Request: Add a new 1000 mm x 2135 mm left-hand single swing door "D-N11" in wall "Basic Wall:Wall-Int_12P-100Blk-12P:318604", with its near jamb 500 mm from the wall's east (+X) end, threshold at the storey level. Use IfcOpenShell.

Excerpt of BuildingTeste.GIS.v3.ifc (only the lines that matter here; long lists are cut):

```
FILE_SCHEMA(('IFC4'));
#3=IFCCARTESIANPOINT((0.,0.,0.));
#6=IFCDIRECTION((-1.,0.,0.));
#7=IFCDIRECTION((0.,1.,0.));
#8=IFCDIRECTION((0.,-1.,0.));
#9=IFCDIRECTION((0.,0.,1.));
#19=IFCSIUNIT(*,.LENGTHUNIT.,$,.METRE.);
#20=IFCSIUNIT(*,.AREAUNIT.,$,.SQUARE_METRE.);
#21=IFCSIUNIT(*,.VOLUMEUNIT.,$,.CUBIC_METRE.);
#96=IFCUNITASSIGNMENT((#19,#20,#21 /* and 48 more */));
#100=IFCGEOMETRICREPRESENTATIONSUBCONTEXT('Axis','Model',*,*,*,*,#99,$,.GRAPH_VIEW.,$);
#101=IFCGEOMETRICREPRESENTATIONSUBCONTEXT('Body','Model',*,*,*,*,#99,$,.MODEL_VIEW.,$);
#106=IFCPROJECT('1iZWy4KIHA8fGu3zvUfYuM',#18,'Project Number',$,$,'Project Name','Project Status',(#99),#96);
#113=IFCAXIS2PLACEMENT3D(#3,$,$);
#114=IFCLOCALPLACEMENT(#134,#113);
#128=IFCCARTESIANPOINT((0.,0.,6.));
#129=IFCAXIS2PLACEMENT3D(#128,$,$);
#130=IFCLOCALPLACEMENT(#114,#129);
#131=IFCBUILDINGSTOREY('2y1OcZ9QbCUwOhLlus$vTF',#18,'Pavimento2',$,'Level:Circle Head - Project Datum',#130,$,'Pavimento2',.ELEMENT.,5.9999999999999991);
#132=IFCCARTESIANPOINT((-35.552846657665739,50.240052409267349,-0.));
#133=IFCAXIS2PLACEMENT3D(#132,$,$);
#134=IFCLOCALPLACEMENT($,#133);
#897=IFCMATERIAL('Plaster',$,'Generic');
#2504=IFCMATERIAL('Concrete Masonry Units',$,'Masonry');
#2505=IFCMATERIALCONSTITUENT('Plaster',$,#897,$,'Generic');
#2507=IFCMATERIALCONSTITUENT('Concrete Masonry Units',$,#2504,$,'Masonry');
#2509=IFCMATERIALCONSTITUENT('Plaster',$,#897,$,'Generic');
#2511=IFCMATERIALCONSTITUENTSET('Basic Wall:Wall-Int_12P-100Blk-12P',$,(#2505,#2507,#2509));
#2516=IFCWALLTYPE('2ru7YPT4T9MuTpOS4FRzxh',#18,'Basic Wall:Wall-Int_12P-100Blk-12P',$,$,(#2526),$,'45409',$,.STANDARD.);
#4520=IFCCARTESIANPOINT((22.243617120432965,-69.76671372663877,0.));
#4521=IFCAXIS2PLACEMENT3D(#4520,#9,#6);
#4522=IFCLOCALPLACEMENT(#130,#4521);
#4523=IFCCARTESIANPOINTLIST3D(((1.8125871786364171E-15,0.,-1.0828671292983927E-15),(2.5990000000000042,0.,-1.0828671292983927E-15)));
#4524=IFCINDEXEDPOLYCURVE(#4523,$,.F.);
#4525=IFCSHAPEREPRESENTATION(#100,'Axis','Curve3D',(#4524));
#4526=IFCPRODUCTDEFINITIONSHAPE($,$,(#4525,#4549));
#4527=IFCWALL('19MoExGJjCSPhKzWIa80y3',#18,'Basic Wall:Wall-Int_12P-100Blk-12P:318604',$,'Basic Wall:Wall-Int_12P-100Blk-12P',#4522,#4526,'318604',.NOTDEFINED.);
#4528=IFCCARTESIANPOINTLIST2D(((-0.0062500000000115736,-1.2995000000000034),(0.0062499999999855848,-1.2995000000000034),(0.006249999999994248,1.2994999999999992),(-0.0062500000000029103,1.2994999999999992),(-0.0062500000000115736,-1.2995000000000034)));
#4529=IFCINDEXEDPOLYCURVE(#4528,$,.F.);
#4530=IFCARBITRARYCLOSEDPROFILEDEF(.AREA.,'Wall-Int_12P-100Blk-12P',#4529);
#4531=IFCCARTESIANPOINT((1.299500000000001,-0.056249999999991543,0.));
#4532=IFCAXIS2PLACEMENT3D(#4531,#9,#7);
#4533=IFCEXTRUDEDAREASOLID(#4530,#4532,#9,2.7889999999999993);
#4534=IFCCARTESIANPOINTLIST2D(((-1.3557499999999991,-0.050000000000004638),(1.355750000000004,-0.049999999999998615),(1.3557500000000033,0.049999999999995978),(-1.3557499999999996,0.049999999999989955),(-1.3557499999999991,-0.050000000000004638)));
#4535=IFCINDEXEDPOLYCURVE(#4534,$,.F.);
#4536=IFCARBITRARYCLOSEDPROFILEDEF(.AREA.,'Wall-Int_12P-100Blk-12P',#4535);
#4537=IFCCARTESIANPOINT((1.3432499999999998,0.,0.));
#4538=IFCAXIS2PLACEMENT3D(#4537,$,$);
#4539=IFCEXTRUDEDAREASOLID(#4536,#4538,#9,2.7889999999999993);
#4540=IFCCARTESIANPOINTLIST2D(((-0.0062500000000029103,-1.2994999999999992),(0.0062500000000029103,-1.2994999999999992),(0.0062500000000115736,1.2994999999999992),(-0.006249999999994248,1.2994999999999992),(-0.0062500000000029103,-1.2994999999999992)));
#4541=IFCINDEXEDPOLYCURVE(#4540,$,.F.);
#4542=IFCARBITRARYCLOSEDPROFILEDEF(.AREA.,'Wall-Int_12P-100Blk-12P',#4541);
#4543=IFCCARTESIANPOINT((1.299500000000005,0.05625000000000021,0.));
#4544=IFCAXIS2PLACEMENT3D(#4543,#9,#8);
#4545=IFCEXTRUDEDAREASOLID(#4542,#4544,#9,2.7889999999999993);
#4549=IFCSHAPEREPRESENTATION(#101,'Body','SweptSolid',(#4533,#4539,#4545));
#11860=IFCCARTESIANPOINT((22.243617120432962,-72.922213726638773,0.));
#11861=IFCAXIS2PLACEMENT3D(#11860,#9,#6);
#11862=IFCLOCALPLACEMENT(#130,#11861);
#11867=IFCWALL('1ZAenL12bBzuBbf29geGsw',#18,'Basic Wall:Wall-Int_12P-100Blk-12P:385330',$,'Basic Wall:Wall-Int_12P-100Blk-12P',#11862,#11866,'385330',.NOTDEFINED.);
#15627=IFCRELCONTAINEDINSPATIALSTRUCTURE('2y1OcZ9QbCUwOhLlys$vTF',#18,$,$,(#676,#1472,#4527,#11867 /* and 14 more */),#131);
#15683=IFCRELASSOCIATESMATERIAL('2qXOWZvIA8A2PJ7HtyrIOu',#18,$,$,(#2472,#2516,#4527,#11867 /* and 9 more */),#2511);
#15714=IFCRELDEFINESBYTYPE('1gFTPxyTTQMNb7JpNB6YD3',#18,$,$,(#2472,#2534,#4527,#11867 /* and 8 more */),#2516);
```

```python
import numpy as np
import ifcopenshell
import ifcopenshell.api.feature
import ifcopenshell.api.geometry
import ifcopenshell.api.root
import ifcopenshell.api.spatial
import ifcopenshell.geom
import ifcopenshell.util.element
import ifcopenshell.util.placement
import ifcopenshell.util.representation
import ifcopenshell.util.shape
import ifcopenshell.util.unit

model = ifcopenshell.open("BuildingTeste.GIS.v3.ifc")
unit_scale = ifcopenshell.util.unit.calculate_unit_scale(model)
settings = ifcopenshell.geom.settings()


def volume(element):
    """Net volume in cubic metres, openings subtracted."""
    shape = ifcopenshell.geom.create_shape(settings, element)
    return ifcopenshell.util.shape.get_volume(shape.geometry)


wall = model.by_guid("19MoExGJjCSPhKzWIa80y3")
storey = ifcopenshell.util.element.get_container(wall, ifc_class="IfcBuildingStorey")
context = ifcopenshell.util.representation.get_context(model, "Model", "Body", "MODEL_VIEW")
before = volume(wall)

width, height, from_end, sill = 1, 2.135, 0.5, 0.0  # metres

# The wall runs along its own X axis, and the end named is its -X end.
wall_shape = ifcopenshell.geom.create_shape(settings, wall)
x, y, z = ifcopenshell.util.shape.get_vertices(wall_shape.geometry).T
start = x.min() + from_end
face, thickness = float(y.min()), float(y.max() - y.min())
wall_matrix = ifcopenshell.util.placement.get_local_placement(wall.ObjectPlacement)
level = ifcopenshell.util.placement.get_local_placement(storey.ObjectPlacement)[2, 3]


def in_wall(x, y):
    """Placement at x, y metres in the wall's axes, at sill height."""
    matrix = wall_matrix.copy()
    matrix[:, 3] = wall_matrix @ np.array([x / unit_scale, y / unit_scale, 0.0, 1.0])
    matrix[2, 3] = level + sill / unit_scale
    return matrix


# Opening: a box that overshoots both wall faces by 50 mm.
opening = ifcopenshell.api.root.create_entity(model, ifc_class="IfcOpeningElement", predefined_type="OPENING")
box = ifcopenshell.api.geometry.add_wall_representation(
    model, context=context, length=width, height=height, thickness=thickness + 0.1
)
ifcopenshell.api.geometry.assign_representation(model, product=opening, representation=box)
ifcopenshell.api.geometry.edit_object_placement(model, product=opening, matrix=in_wall(start, face - 0.05), is_si=False)
ifcopenshell.api.feature.add_feature(model, feature=opening, element=wall)

door = ifcopenshell.api.root.create_entity(model, ifc_class="IfcDoor", name="D-N11", predefined_type="DOOR")
door.OverallWidth, door.OverallHeight = width / unit_scale, height / unit_scale
door.OperationType = "SINGLE_SWING_LEFT"
body = ifcopenshell.api.geometry.add_door_representation(
    model,
    context=context,
    overall_width=door.OverallWidth,
    overall_height=door.OverallHeight,
    operation_type="SINGLE_SWING_LEFT",
    lining_properties={"LiningDepth": thickness / unit_scale, "ThresholdDepth": thickness / unit_scale},
)
ifcopenshell.api.geometry.assign_representation(model, product=door, representation=body)
ifcopenshell.api.spatial.assign_container(model, products=[door], relating_structure=storey)
ifcopenshell.api.feature.add_filling(model, opening=opening, element=door)

# The lining spans the wall, so the door starts at the wall face.
ifcopenshell.api.geometry.edit_object_placement(model, product=door, matrix=in_wall(start, face), is_si=False)

after = volume(wall)

print(f"wall volume {before:.3f} -> {after:.3f} m3")

model.write("BuildingTeste.GIS.v3_edited.ifc")
```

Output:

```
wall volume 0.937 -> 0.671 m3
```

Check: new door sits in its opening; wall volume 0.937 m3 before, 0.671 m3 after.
